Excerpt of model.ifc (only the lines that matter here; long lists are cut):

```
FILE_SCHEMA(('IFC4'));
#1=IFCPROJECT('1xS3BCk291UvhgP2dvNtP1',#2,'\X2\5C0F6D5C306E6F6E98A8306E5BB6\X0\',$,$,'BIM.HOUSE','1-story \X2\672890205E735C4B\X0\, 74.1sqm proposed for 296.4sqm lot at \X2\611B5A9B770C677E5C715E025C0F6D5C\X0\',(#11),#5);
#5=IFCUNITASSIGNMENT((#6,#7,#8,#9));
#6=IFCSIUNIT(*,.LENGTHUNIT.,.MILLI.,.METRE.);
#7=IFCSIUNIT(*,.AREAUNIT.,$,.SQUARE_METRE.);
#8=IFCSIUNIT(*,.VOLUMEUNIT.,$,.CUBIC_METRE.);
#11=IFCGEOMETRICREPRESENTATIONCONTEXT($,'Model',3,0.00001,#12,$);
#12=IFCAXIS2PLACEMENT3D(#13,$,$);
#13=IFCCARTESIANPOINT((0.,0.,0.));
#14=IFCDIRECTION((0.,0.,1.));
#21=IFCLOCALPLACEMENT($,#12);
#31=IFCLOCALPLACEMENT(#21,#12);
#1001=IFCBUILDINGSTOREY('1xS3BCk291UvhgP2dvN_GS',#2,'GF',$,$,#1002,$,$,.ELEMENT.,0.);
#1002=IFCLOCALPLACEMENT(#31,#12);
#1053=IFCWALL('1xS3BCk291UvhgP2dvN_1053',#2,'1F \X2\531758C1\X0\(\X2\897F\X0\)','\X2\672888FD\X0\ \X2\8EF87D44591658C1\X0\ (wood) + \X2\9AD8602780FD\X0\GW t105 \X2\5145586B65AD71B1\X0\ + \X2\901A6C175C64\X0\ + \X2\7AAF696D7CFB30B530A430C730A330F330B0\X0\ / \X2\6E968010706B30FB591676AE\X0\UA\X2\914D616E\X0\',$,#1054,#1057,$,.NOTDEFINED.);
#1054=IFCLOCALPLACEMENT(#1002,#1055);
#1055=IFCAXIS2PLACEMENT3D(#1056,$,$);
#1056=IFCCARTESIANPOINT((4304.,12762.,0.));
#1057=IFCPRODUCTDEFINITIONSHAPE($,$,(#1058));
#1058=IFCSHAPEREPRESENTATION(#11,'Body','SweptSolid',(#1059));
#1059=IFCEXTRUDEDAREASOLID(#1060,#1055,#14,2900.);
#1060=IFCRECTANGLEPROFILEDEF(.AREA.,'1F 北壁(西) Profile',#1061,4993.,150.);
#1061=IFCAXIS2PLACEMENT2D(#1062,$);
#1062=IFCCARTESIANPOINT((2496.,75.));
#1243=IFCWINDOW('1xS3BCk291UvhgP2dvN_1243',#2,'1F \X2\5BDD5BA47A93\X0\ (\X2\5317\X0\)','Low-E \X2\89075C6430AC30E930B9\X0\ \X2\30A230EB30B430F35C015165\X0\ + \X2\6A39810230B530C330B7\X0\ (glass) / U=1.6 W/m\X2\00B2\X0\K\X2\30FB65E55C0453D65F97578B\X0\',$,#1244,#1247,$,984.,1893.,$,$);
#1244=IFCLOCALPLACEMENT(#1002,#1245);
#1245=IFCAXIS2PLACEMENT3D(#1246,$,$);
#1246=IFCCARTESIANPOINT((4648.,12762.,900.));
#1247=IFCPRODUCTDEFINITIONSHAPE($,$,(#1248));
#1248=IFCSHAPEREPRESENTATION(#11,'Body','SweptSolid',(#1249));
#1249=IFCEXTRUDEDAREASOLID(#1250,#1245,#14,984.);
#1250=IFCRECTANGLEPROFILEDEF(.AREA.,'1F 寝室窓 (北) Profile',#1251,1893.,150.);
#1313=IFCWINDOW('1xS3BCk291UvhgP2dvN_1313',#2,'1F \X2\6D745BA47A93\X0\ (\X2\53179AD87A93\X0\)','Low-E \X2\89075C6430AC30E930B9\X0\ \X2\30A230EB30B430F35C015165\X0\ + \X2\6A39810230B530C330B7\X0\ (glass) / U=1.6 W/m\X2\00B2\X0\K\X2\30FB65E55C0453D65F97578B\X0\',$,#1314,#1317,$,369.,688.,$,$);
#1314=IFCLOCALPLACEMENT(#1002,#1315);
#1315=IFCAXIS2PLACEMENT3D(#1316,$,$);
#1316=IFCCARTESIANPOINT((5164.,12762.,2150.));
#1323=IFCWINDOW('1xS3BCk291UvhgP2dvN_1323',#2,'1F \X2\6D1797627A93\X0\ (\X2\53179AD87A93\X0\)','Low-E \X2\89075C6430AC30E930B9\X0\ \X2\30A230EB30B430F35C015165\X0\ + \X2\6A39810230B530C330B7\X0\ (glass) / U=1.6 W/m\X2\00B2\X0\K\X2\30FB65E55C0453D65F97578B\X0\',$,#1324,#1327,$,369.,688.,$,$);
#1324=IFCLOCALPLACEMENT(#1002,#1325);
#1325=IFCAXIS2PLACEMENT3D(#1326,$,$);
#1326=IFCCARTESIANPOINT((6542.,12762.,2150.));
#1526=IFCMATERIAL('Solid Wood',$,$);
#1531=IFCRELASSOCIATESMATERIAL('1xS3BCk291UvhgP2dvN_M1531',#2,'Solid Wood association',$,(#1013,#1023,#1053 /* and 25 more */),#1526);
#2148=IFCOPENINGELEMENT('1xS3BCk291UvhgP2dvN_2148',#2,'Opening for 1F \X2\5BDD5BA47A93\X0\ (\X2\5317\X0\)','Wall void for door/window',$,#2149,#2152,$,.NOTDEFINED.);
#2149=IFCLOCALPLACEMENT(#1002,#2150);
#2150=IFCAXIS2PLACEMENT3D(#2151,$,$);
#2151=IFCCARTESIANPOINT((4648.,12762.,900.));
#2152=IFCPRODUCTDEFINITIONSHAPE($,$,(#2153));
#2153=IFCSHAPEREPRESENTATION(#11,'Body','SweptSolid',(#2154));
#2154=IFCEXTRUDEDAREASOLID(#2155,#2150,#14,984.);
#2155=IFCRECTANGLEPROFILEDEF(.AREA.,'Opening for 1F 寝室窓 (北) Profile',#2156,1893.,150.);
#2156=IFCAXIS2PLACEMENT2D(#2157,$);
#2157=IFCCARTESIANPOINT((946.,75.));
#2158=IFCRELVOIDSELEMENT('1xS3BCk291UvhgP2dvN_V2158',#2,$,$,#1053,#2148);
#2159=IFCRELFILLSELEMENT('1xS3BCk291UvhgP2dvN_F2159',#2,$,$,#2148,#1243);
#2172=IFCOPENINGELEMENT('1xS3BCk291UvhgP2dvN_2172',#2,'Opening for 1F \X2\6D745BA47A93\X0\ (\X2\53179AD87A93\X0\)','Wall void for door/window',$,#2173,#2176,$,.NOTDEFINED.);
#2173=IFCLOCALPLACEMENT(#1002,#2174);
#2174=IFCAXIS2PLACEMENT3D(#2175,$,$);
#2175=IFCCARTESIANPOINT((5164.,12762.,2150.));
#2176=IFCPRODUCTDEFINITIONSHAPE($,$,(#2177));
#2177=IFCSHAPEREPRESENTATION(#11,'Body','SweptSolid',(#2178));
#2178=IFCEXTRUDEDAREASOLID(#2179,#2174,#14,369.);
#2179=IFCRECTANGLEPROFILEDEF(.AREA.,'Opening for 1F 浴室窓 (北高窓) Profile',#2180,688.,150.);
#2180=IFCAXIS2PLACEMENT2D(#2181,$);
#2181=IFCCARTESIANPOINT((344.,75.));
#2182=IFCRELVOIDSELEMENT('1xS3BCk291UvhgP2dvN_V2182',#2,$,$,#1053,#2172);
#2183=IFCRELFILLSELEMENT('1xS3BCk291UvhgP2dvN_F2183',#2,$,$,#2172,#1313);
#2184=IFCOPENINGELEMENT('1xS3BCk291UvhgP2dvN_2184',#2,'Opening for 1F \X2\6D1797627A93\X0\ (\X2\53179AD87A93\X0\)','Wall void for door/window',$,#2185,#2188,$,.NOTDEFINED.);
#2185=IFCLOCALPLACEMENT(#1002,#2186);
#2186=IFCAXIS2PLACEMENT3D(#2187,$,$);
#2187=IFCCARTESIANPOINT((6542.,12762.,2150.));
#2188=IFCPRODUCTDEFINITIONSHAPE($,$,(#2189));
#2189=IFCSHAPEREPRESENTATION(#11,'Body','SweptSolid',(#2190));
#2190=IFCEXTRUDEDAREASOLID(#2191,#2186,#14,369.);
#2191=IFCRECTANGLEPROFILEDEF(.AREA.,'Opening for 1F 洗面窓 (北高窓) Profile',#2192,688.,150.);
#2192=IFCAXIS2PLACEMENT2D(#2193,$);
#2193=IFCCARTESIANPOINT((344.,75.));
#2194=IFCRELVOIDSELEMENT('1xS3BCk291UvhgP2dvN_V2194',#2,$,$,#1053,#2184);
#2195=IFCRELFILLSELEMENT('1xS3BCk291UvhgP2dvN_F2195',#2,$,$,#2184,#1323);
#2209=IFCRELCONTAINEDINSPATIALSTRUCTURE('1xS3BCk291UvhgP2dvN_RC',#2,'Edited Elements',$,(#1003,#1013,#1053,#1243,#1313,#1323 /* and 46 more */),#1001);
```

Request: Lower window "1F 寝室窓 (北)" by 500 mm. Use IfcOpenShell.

```python
import numpy as np
import ifcopenshell
import ifcopenshell.api.geometry
import ifcopenshell.util.placement
import ifcopenshell.util.unit

model = ifcopenshell.open("model.ifc")
unit_scale = ifcopenshell.util.unit.calculate_unit_scale(model)

window = model.by_guid("1xS3BCk291UvhgP2dvN_1243")
opening = window.FillsVoids[0].RelatingOpeningElement
dz = -500.0

shift = np.array([0.0, 0.0, dz])
# The window is not placed relative to its opening, so move both.
for product in (opening, window):
    matrix = ifcopenshell.util.placement.get_local_placement(product.ObjectPlacement)
    matrix[:3, 3] += shift
    ifcopenshell.api.geometry.edit_object_placement(model, product=product, matrix=matrix, is_si=False)

print(f"moved by {dz * unit_scale:+.3f} m")

model.write("model_rev.ifc")
```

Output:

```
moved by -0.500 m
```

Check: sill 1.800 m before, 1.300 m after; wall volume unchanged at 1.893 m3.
